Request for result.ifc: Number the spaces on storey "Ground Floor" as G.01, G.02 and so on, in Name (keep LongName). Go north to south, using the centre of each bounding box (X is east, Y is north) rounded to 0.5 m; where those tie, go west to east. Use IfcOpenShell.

First a look at what the model holds.

```python
import ifcopenshell
import ifcopenshell.util.element
import ifcopenshell.util.placement

model = ifcopenshell.open("result.ifc")
print(model.schema)
storey = next(s for s in model.by_type("IfcBuildingStorey") if s.Name == "Ground Floor")
spaces = [e for e in ifcopenshell.util.element.get_decomposition(storey) if e.is_a("IfcSpace")]
for e in sorted(spaces, key=lambda e: e.id()):
    origin = ifcopenshell.util.placement.get_local_placement(e.ObjectPlacement)[:3, 3]
    print(e.id(), e.Name, e.LongName, origin.round(2) + 0.0, sep=" | ")
```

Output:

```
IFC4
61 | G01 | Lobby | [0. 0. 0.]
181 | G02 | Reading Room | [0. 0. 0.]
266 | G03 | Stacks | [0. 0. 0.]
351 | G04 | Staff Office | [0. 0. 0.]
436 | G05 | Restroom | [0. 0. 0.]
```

```python
import ifcopenshell
import ifcopenshell.geom
import ifcopenshell.util.element
import ifcopenshell.util.shape

model = ifcopenshell.open("result.ifc")
settings = ifcopenshell.geom.settings()
settings.set("use-world-coords", True)


def centre(element):
    shape = ifcopenshell.geom.create_shape(settings, element)
    return ifcopenshell.util.shape.get_bbox_centroid(shape.geometry)


storey = next(s for s in model.by_type("IfcBuildingStorey") if s.Name == "Ground Floor")
spaces = [e for e in ifcopenshell.util.element.get_decomposition(storey) if e.is_a("IfcSpace")]

# Insertion points can sit at a corner or the storey origin, so sort by the geometry (in metres).
centres = {e: centre(e) for e in spaces}
spaces.sort(key=lambda e: (-round(centres[e][1] / 0.5), centres[e][0]))

for i, e in enumerate(spaces, start=1):
    number = f"G.{i:02d}"
    e.Name = number
    print(e.id(), number)

model.write("result_v2.ifc")
```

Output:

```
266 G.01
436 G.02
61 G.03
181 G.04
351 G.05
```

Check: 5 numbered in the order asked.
